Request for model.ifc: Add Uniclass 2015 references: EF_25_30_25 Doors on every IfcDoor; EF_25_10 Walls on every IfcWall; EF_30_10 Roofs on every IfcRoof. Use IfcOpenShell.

First a look at what the model holds.

```python
import ifcopenshell

model = ifcopenshell.open("model.ifc")
print(model.schema)
print("classifications:", [c.Name for c in model.by_type("IfcClassification")])
for ifc_class in ("IfcDoor", "IfcRoof", "IfcStair", "IfcWall", "IfcWindow"):
    print(ifc_class, len(model.by_type(ifc_class)))
```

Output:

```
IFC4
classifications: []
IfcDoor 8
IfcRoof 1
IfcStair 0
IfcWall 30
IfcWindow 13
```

```python
import ifcopenshell
import ifcopenshell.api.classification

model = ifcopenshell.open("model.ifc")

system = ifcopenshell.api.classification.add_classification(model, classification="Uniclass 2015")

codes = {
    "IfcDoor": ("EF_25_30_25", "Doors"),
    "IfcWall": ("EF_25_10", "Walls"),
    "IfcRoof": ("EF_30_10", "Roofs"),
}
for ifc_class, (code, name) in codes.items():
    products = model.by_type(ifc_class)
    ifcopenshell.api.classification.add_reference(
        model, products=products, classification=system, identification=code, name=name
    )
    print(code, len(products))

model.write("model-out.ifc")
```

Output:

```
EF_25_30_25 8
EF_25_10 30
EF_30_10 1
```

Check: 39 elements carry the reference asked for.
